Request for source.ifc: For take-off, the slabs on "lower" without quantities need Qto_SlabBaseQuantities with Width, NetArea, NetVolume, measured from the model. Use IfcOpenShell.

First a look at what the model holds.

```python
import ifcopenshell
import ifcopenshell.util.element
import ifcopenshell.util.unit

model = ifcopenshell.open("source.ifc")
print(model.schema)
for unit_type in ("LENGTHUNIT", "AREAUNIT", "VOLUMEUNIT"):
    print(unit_type, ifcopenshell.util.unit.calculate_unit_scale(model, unit_type))
storey = next(s for s in model.by_type("IfcBuildingStorey") if s.Name == "lower")
slabs = [e for e in ifcopenshell.util.element.get_decomposition(storey) if e.is_a("IfcSlab")]
for e in sorted(slabs, key=lambda e: e.id()):
    print(e.id(), e.is_a(), e.Name, list(ifcopenshell.util.element.get_psets(e, qtos_only=True)), sep=" | ")
```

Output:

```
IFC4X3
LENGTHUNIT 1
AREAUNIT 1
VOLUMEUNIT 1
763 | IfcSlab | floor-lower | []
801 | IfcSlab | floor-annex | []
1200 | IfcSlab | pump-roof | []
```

```python
import ifcopenshell
import ifcopenshell.api.pset
import ifcopenshell.geom
import ifcopenshell.util.element
import ifcopenshell.util.shape
import ifcopenshell.util.unit

model = ifcopenshell.open("source.ifc")
unit_scale = ifcopenshell.util.unit.calculate_unit_scale(model)
area_scale = ifcopenshell.util.unit.calculate_unit_scale(model, "AREAUNIT")
volume_scale = ifcopenshell.util.unit.calculate_unit_scale(model, "VOLUMEUNIT")
settings = ifcopenshell.geom.settings()

storey = next(s for s in model.by_type("IfcBuildingStorey") if s.Name == "lower")
slabs = [e for e in ifcopenshell.util.element.get_decomposition(storey) if e.is_a("IfcSlab")]

for e in sorted(slabs, key=lambda e: e.id()):
    if ifcopenshell.util.element.get_psets(e, qtos_only=True, should_inherit=False):
        continue
    # Geometry comes back in metres, in the element's own axes.
    shape = ifcopenshell.geom.create_shape(settings, e)
    values = {
        "Width": ifcopenshell.util.shape.get_z(shape.geometry) / unit_scale,
        "NetArea": ifcopenshell.util.shape.get_footprint_area(shape.geometry) / area_scale,
        "NetVolume": ifcopenshell.util.shape.get_volume(shape.geometry) / volume_scale,
    }
    qto = ifcopenshell.api.pset.add_qto(model, product=e, name="Qto_SlabBaseQuantities")
    ifcopenshell.api.pset.edit_qto(model, qto=qto, properties=values)
    print(e.id(), {k: round(v, 3) for k, v in values.items()})

model.write("source-out.ifc")
```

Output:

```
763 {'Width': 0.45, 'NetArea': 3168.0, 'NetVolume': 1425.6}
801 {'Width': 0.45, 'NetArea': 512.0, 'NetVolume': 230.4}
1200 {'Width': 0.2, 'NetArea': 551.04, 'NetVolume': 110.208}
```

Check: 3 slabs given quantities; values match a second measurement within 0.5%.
